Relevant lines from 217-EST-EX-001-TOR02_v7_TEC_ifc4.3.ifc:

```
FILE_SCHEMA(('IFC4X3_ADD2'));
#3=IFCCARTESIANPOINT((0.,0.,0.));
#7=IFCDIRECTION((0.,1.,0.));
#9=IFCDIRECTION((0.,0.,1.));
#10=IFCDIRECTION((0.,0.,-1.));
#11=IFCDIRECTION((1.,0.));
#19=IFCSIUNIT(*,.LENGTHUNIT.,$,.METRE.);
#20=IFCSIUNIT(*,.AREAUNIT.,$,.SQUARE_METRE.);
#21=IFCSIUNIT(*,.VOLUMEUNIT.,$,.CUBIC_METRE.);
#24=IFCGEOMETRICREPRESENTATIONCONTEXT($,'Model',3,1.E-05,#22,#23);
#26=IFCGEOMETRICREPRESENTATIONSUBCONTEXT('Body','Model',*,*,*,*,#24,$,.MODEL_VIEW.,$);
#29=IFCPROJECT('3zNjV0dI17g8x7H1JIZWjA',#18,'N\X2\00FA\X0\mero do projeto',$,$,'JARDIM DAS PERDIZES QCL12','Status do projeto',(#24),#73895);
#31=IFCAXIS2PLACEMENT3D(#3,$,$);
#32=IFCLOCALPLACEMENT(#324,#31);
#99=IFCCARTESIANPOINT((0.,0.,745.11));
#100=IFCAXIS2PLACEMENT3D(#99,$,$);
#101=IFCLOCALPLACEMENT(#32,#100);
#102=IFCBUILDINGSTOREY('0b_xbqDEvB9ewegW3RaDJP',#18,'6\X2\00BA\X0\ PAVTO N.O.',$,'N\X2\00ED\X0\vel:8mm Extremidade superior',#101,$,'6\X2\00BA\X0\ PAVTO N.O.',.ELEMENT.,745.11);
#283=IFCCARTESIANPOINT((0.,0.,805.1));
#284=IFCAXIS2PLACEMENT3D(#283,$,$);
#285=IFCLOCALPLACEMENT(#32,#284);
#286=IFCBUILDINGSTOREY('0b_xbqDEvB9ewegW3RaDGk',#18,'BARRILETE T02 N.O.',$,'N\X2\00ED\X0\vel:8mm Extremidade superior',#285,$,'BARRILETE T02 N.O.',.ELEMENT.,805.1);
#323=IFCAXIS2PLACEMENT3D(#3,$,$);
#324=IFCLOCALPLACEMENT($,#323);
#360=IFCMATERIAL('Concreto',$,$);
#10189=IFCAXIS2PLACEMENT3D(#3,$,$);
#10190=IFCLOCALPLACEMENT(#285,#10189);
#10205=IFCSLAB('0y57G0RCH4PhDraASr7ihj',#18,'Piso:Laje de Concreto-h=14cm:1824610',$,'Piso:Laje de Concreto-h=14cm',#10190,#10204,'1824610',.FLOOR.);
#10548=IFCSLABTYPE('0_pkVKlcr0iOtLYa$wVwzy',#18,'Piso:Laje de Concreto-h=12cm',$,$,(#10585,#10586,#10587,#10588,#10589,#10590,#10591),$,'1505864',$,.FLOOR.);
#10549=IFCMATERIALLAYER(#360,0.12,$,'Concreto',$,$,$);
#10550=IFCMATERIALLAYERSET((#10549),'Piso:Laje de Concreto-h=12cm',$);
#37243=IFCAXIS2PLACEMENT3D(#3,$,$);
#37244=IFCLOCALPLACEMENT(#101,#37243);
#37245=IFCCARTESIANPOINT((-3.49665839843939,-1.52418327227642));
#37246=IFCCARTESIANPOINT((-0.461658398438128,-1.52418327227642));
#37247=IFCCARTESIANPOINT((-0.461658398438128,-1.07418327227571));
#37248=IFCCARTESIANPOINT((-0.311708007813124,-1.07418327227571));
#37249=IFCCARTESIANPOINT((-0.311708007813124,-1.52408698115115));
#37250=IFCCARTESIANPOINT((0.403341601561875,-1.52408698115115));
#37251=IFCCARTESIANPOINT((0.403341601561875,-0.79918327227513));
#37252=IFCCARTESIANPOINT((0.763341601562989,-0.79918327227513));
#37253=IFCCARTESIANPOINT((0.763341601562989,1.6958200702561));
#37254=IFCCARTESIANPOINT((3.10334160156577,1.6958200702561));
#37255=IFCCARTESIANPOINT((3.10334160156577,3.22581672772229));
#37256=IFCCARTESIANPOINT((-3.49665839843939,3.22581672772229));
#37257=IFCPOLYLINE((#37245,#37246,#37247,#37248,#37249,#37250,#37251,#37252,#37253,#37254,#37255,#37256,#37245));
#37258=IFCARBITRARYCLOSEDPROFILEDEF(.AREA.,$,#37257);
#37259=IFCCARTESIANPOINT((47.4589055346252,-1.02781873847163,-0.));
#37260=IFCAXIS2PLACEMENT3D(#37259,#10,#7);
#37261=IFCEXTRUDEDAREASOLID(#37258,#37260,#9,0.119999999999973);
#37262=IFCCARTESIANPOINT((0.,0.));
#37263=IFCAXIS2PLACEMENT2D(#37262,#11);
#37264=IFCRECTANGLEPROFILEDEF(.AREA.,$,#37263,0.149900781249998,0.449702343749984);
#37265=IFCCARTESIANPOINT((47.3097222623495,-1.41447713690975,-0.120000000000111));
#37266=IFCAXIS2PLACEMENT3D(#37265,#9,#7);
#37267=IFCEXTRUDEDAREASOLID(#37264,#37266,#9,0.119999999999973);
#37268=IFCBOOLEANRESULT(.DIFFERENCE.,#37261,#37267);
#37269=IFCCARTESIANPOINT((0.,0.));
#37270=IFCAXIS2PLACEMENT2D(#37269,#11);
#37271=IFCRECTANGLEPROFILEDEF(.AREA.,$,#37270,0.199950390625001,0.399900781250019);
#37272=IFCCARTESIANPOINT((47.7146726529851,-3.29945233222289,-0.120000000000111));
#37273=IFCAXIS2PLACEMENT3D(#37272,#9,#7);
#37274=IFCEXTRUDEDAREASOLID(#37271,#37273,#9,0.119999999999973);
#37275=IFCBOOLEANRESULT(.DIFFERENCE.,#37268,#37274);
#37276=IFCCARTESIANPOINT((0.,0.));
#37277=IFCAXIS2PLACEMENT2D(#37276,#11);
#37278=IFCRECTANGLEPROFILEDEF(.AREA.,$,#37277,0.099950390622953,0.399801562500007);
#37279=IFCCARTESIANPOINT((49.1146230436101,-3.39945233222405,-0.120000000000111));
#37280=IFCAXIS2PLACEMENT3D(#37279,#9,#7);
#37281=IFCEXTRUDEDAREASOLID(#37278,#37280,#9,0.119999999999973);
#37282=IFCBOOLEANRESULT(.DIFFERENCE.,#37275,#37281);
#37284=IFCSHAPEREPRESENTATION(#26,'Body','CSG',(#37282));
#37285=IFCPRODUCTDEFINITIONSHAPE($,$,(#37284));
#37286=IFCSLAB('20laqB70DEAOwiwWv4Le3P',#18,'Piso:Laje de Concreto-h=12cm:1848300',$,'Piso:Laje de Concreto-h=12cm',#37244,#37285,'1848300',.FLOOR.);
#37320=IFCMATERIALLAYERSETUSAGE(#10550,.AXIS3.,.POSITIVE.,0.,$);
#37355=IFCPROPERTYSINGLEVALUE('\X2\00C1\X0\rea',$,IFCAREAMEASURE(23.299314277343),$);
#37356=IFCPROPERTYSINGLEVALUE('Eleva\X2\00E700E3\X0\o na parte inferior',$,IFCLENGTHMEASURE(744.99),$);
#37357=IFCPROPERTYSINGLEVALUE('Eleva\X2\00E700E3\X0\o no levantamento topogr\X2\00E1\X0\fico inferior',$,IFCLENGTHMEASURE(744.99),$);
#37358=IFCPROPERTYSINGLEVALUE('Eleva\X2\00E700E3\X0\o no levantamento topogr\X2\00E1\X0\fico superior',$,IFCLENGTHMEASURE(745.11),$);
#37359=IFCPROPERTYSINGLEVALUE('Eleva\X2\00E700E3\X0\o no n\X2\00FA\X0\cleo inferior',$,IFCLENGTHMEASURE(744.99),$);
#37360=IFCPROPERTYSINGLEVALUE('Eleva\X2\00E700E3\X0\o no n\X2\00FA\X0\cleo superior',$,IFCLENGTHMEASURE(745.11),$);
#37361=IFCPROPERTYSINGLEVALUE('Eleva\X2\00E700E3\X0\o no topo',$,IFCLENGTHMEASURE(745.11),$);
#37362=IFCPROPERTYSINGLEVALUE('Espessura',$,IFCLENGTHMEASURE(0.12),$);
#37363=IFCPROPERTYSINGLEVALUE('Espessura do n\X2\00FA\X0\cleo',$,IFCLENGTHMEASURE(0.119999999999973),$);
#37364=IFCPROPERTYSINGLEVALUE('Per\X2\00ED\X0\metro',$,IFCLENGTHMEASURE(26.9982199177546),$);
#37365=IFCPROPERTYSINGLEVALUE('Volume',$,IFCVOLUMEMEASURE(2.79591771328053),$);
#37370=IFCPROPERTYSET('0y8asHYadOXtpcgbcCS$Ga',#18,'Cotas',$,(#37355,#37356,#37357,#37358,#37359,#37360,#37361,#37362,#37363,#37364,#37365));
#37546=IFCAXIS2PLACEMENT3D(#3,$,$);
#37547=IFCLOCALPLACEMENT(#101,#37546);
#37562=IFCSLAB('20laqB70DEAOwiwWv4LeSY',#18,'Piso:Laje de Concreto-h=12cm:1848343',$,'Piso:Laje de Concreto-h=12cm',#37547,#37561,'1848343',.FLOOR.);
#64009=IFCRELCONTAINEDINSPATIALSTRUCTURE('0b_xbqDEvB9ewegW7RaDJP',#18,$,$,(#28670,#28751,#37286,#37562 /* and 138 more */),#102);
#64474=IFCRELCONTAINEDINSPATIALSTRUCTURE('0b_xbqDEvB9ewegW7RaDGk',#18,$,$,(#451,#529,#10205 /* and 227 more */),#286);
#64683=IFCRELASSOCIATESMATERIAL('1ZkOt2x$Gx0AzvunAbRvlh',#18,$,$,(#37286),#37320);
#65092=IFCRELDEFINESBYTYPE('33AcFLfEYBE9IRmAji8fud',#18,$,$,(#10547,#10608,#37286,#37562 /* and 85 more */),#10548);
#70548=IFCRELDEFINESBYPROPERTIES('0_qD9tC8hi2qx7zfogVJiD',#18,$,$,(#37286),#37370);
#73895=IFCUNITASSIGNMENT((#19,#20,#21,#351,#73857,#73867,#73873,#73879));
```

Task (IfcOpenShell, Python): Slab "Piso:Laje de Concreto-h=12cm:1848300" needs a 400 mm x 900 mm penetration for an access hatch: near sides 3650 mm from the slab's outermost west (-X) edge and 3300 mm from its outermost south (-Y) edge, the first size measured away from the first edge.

```python
import numpy as np
import ifcopenshell
import ifcopenshell.api.feature
import ifcopenshell.api.geometry
import ifcopenshell.api.pset
import ifcopenshell.api.root
import ifcopenshell.geom
import ifcopenshell.util.element
import ifcopenshell.util.placement
import ifcopenshell.util.representation
import ifcopenshell.util.shape
import ifcopenshell.util.unit

model = ifcopenshell.open("217-EST-EX-001-TOR02_v7_TEC_ifc4.3.ifc")
unit_scale = ifcopenshell.util.unit.calculate_unit_scale(model)
area_scale = ifcopenshell.util.unit.calculate_unit_scale(model, "AREAUNIT")
volume_scale = ifcopenshell.util.unit.calculate_unit_scale(model, "VOLUMEUNIT")
settings = ifcopenshell.geom.settings()


def volume(element):
    """Net volume in cubic metres, openings subtracted."""
    shape = ifcopenshell.geom.create_shape(settings, element)
    return ifcopenshell.util.shape.get_volume(shape.geometry)


slab = model.by_guid("20laqB70DEAOwiwWv4Le3P")
before = volume(slab)

# Extent in the slab's own axes, in metres. The edges named are its -X and -Y sides.
slab_shape = ifcopenshell.geom.create_shape(settings, slab)
vertices = ifcopenshell.util.shape.get_vertices(slab_shape.geometry)
x_min, y_min, bottom = vertices.min(axis=0)
top = vertices[:, 2].max()

opening = ifcopenshell.api.root.create_entity(model, ifc_class="IfcOpeningElement", name="Access hatch opening", predefined_type="OPENING")
context = ifcopenshell.util.representation.get_context(model, "Model", "Body", "MODEL_VIEW")
width, depth = 0.4, 0.9
outline = [(0.0, 0.0), (width, 0.0), (width, depth), (0.0, depth), (0.0, 0.0)]
# Overshoot both faces by 50 mm so the cut is clean.
shape = ifcopenshell.api.geometry.add_slab_representation(
    model, context=context, depth=top - bottom + 0.1, polyline=outline
)
ifcopenshell.api.geometry.assign_representation(model, product=opening, representation=shape)

matrix = ifcopenshell.util.placement.get_local_placement(slab.ObjectPlacement)
matrix[:, 3] = matrix @ np.append(np.array([x_min + 3.65, y_min + 3.3, bottom - 0.05]) / unit_scale, 1.0)
ifcopenshell.api.geometry.edit_object_placement(model, product=opening, matrix=matrix, is_si=False)
ifcopenshell.api.feature.add_feature(model, feature=opening, element=slab)

after = volume(slab)

# Update the slab's stored quantities.
pset = model.by_id(ifcopenshell.util.element.get_pset(slab, "Cotas", should_inherit=False)["id"])
ifcopenshell.api.pset.edit_pset(model, pset=pset, properties={
    "Área": model.create_entity("IfcAreaMeasure", after / (top - bottom) / area_scale),
    "Volume": model.create_entity("IfcVolumeMeasure", after / volume_scale),
})

print(f"slab volume {before:.3f} -> {after:.3f} m3")

model.write("217-EST-EX-001-TOR02_v7_TEC_ifc4.3_v2.ifc")
```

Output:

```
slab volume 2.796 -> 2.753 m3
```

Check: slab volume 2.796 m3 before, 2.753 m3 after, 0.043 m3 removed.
